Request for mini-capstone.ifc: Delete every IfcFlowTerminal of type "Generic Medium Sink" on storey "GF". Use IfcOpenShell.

First a look at what the model holds.

```python
import ifcopenshell
import ifcopenshell.util.element

model = ifcopenshell.open("mini-capstone.ifc")
print(model.schema)
storey = next(s for s in model.by_type("IfcBuildingStorey") if s.Name == "GF")
terminals = [e for e in ifcopenshell.util.element.get_decomposition(storey) if e.is_a("IfcFlowTerminal")]
seen = {}
for e in terminals:
    element_type = ifcopenshell.util.element.get_type(e)
    name = element_type.Name if element_type not in (None, e) else None
    seen[name] = seen.get(name, 0) + 1
for name, count in sorted(seen.items(), key=str):
    print(count, "x", name)
```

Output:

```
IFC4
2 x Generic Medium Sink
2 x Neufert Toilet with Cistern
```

```python
import ifcopenshell
import ifcopenshell.api.root
import ifcopenshell.util.element

model = ifcopenshell.open("mini-capstone.ifc")

storey = next(s for s in model.by_type("IfcBuildingStorey") if s.Name == "GF")
terminals = [e for e in ifcopenshell.util.element.get_decomposition(storey) if e.is_a("IfcFlowTerminal")]
targets = [e for e in terminals if (t := ifcopenshell.util.element.get_type(e)) not in (None, e) and t.Name == "Generic Medium Sink"]

for e in targets:
    ifcopenshell.api.root.remove_product(model, product=e)
print(len(targets), "removed")

model.write("mini-capstone_edited.ifc")
```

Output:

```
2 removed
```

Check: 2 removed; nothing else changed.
